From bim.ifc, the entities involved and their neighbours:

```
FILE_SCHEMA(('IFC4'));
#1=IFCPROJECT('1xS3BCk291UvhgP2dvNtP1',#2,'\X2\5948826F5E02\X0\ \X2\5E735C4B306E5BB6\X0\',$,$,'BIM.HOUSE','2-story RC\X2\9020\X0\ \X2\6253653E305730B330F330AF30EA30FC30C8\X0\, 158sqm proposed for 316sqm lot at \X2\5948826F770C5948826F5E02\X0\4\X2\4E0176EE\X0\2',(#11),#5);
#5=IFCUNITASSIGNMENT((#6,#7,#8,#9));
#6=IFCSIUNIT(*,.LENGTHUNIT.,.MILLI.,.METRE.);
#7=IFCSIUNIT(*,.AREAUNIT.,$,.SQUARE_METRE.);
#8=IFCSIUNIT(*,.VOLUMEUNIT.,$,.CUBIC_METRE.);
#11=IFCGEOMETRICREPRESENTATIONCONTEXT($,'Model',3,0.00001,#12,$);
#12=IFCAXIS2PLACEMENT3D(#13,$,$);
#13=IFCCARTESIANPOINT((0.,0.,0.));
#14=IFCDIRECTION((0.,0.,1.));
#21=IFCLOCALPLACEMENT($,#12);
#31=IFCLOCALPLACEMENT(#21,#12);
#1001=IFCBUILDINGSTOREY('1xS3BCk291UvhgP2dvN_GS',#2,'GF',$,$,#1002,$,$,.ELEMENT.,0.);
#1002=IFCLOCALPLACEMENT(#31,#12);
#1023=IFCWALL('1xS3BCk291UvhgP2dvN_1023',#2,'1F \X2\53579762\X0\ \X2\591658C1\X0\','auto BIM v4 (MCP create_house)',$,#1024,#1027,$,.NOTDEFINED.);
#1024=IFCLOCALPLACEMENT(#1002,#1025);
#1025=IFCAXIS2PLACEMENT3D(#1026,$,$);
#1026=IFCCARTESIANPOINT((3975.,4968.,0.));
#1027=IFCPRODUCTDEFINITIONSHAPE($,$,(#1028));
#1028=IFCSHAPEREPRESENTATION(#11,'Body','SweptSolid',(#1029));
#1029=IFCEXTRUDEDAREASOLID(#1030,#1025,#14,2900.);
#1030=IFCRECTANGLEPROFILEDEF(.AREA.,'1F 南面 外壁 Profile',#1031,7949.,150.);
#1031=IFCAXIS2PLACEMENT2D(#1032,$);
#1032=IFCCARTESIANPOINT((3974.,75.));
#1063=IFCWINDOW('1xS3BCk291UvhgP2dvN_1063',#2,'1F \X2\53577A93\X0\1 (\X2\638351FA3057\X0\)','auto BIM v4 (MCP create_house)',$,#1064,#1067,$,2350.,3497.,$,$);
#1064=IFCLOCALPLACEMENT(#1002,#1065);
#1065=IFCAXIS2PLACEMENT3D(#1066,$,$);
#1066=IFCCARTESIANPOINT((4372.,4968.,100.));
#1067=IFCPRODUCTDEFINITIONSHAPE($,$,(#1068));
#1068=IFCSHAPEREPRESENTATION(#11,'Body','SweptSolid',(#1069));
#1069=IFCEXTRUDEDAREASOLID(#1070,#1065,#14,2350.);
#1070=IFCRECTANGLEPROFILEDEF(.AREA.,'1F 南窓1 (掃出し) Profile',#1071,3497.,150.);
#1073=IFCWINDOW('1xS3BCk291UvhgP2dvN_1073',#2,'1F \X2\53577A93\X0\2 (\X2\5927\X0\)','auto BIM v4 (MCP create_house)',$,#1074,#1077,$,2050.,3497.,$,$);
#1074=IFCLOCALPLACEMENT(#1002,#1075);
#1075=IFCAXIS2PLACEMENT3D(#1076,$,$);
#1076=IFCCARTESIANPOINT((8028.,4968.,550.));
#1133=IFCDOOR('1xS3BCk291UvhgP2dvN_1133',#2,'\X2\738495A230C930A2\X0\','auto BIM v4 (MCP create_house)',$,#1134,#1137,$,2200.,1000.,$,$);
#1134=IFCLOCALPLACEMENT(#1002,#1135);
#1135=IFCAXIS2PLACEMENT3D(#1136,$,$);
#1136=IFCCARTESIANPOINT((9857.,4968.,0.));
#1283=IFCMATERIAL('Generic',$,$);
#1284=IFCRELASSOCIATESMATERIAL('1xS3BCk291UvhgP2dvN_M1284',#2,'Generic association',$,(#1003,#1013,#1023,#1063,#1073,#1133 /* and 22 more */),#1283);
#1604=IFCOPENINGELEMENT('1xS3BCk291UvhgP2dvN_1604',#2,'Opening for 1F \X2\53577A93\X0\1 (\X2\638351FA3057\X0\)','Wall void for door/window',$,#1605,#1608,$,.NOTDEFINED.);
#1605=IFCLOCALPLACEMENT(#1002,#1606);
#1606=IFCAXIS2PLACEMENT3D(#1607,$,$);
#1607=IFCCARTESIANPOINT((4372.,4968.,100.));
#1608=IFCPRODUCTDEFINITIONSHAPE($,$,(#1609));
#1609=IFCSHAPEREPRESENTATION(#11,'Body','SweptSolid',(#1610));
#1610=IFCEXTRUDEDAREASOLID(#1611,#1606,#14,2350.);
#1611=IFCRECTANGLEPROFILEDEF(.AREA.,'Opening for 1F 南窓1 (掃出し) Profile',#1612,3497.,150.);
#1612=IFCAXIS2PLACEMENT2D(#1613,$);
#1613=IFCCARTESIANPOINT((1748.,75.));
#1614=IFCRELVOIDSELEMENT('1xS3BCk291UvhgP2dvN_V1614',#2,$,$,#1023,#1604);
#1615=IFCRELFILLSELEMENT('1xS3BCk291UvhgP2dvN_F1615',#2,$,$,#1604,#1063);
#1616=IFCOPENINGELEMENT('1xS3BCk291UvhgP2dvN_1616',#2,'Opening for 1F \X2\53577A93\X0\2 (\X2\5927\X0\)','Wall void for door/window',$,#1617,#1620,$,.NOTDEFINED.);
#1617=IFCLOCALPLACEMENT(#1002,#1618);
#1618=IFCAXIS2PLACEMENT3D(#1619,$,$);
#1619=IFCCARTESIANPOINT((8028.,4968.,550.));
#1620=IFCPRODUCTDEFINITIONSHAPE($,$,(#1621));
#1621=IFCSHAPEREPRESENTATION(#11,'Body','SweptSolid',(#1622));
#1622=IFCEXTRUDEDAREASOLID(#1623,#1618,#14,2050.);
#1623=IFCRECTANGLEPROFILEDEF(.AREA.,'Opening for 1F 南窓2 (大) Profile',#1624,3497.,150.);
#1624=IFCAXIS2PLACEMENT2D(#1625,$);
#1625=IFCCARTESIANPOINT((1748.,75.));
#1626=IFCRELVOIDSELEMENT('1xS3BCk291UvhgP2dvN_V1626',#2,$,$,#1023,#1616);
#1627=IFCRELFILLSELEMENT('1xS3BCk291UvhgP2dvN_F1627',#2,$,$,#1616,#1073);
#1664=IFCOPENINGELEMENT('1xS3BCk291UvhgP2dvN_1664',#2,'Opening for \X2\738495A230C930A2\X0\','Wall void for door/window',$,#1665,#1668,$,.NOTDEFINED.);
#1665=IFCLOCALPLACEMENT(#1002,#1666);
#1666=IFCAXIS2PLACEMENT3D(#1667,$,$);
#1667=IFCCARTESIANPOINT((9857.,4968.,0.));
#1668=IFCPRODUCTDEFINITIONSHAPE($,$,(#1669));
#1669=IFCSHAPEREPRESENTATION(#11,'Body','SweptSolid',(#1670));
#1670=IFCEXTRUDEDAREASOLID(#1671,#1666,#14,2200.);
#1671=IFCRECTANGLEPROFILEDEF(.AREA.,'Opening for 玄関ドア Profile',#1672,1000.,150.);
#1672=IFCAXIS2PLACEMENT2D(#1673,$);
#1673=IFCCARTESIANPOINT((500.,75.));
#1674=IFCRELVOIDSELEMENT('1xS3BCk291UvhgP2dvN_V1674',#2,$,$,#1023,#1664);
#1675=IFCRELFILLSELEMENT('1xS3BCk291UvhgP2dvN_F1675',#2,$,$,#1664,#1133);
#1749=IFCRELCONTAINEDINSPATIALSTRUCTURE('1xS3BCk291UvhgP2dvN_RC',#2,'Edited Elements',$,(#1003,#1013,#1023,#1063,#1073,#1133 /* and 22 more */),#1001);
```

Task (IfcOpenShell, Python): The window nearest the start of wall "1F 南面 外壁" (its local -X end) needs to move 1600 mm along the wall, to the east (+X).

```python
import ifcopenshell
import ifcopenshell.api.geometry
import ifcopenshell.util.placement
import ifcopenshell.util.unit

model = ifcopenshell.open("bim.ifc")
unit_scale = ifcopenshell.util.unit.calculate_unit_scale(model)

window = model.by_guid("1xS3BCk291UvhgP2dvN_1063")
opening = window.FillsVoids[0].RelatingOpeningElement
wall = opening.VoidsElements[0].RelatingBuildingElement

wall_matrix = ifcopenshell.util.placement.get_local_placement(wall.ObjectPlacement)
shift = wall_matrix[:3, 0] * 1.6 / unit_scale
before = ifcopenshell.util.placement.get_local_placement(window.ObjectPlacement)[:3, 3].copy()

# The window is not placed relative to its opening, so move both.
for product in (opening, window):
    matrix = ifcopenshell.util.placement.get_local_placement(product.ObjectPlacement)
    matrix[:3, 3] += shift
    ifcopenshell.api.geometry.edit_object_placement(model, product=product, matrix=matrix, is_si=False)

after = ifcopenshell.util.placement.get_local_placement(window.ObjectPlacement)[:3, 3]
print("window moved by", (after - before).round(3) + 0.0)

model.write("bim_rev.ifc")
```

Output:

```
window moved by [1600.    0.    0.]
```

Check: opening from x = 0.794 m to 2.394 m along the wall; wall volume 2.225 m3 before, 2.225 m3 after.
